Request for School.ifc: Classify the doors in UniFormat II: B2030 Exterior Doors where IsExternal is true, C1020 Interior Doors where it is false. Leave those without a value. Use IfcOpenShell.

First a look at what the model holds.

```python
import ifcopenshell
import ifcopenshell.util.element

model = ifcopenshell.open("School.ifc")
print(model.schema)
print("classifications:", [c.Name for c in model.by_type("IfcClassification")])
values = [ifcopenshell.util.element.get_pset(e, "Pset_DoorCommon", "IsExternal") for e in model.by_type("IfcDoor")]
for value in (True, False, None):
    print("IsExternal", value, values.count(value))
```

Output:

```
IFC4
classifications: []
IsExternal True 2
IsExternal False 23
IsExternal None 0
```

```python
import ifcopenshell
import ifcopenshell.api.classification
import ifcopenshell.util.element

model = ifcopenshell.open("School.ifc")

system = ifcopenshell.api.classification.add_classification(model, classification="UniFormat II")

doors = model.by_type("IfcDoor")
external = {e: ifcopenshell.util.element.get_pset(e, "Pset_DoorCommon", "IsExternal") for e in doors}
for flag, code, name in ((True, "B2030", "Exterior Doors"), (False, "C1020", "Interior Doors")):
    products = [e for e in doors if external[e] is flag]
    ifcopenshell.api.classification.add_reference(
        model, products=products, classification=system, identification=code, name=name
    )
    print(code, len(products))

model.write("School_edited.ifc")
```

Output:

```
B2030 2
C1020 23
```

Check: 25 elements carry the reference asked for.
